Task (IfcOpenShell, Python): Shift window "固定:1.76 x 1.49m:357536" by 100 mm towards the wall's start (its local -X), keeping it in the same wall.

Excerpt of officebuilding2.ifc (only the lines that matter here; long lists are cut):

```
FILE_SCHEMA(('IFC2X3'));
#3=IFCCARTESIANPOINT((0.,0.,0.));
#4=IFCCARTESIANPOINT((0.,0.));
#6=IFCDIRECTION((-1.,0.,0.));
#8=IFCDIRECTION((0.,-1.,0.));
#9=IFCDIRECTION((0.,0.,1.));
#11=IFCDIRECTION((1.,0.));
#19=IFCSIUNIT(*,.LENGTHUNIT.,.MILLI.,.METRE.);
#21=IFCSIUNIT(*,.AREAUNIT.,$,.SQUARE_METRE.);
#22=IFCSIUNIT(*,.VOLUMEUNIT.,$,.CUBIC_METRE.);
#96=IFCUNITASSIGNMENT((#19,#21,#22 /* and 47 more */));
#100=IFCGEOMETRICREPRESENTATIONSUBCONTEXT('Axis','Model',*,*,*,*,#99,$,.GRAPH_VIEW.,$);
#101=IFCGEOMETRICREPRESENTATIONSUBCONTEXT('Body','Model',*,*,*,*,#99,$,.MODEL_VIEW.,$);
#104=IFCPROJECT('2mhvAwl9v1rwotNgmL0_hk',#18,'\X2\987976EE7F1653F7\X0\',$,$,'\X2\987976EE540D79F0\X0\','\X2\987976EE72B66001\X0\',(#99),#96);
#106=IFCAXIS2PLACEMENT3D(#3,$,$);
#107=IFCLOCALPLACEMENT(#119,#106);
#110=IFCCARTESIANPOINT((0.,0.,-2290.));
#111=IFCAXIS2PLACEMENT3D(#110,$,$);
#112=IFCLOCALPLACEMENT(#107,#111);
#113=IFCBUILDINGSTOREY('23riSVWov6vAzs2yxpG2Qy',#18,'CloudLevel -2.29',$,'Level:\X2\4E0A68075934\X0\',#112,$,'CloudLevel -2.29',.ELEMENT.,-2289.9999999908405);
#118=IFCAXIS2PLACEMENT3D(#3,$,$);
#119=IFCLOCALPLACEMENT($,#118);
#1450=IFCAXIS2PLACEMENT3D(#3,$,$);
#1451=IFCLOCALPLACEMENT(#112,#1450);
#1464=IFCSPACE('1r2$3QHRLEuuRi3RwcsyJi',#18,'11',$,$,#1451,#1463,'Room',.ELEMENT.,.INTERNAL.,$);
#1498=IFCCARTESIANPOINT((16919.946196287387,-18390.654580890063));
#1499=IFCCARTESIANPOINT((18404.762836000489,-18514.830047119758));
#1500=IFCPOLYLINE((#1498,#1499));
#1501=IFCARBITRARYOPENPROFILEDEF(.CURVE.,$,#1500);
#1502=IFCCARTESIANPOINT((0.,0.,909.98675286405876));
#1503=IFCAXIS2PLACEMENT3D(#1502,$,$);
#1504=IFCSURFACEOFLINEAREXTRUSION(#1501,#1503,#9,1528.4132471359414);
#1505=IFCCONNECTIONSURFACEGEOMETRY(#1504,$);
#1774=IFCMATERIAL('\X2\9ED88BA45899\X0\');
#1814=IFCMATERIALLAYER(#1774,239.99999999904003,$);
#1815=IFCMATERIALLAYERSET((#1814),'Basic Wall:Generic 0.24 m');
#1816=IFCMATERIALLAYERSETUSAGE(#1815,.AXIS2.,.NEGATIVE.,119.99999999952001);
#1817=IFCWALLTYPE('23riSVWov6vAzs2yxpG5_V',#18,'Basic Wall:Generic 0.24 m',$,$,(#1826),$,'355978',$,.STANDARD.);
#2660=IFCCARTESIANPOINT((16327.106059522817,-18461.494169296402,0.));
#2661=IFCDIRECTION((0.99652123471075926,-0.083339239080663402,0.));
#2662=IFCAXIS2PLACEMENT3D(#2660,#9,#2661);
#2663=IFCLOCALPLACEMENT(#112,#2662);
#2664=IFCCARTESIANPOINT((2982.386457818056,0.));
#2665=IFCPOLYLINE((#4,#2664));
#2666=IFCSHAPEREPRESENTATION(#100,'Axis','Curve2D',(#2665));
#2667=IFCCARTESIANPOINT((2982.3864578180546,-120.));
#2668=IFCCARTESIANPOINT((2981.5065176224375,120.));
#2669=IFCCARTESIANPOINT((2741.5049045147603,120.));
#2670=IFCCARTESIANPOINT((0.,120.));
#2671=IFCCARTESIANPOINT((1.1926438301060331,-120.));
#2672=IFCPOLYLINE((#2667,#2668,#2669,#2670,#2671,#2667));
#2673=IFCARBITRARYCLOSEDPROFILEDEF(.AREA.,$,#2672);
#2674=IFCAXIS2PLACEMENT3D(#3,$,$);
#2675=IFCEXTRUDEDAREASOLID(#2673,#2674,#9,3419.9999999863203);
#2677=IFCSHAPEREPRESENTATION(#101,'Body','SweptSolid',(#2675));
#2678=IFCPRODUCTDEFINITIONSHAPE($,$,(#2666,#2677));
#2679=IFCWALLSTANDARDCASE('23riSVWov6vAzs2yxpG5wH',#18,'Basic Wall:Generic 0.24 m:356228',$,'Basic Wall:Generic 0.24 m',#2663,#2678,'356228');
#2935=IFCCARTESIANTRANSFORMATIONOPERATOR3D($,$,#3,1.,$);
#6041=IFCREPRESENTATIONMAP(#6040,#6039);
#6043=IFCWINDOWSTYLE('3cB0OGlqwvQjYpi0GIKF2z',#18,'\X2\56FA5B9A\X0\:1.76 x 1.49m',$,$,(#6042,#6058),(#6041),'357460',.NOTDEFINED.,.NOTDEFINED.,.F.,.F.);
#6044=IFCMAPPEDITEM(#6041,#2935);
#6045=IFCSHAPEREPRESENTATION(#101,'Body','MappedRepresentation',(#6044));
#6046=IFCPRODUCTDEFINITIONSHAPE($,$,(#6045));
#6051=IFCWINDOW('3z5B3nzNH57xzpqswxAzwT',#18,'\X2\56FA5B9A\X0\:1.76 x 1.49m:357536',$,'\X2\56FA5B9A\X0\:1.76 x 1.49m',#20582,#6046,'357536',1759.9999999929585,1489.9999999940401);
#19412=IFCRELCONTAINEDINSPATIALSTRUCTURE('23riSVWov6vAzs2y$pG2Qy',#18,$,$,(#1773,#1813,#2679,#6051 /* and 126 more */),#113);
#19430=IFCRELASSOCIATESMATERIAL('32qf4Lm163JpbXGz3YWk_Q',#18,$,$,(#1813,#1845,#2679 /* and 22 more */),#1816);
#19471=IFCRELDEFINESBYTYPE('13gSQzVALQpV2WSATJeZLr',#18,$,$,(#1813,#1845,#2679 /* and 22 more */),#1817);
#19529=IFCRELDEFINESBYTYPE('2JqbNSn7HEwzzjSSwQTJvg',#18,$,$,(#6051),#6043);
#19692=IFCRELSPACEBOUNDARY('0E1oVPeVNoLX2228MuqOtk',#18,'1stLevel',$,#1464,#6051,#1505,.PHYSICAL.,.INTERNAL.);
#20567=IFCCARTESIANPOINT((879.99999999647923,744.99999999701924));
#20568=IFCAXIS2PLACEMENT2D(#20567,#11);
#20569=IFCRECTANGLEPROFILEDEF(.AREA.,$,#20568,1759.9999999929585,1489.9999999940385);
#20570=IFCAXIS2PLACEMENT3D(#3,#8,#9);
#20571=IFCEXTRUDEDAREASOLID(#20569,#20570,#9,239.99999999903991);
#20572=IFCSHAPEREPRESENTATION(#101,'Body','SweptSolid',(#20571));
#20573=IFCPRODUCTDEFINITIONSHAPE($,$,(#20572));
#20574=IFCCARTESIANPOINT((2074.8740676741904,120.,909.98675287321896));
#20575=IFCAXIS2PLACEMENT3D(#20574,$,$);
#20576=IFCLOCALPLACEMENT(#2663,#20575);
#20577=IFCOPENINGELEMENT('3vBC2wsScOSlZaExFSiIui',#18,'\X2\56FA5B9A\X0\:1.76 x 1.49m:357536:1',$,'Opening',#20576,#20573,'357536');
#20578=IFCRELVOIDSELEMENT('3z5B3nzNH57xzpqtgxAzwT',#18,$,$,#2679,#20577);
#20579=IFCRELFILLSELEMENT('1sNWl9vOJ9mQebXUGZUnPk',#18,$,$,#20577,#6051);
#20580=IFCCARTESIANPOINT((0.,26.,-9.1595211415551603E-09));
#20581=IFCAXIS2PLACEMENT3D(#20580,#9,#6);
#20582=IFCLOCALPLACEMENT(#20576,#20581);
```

```python
import numpy as np
import ifcopenshell
import ifcopenshell.api.geometry
import ifcopenshell.util.placement
import ifcopenshell.util.unit

model = ifcopenshell.open("officebuilding2.ifc")
unit_scale = ifcopenshell.util.unit.calculate_unit_scale(model)

window = model.by_guid("3z5B3nzNH57xzpqswxAzwT")
opening = window.FillsVoids[0].RelatingOpeningElement
wall = opening.VoidsElements[0].RelatingBuildingElement

wall_matrix = ifcopenshell.util.placement.get_local_placement(wall.ObjectPlacement)
shift = wall_matrix[:3, 0] * -0.1 / unit_scale
before = ifcopenshell.util.placement.get_local_placement(window.ObjectPlacement)[:3, 3].copy()

# The window is placed relative to its opening, so it follows when the opening moves.
matrix = ifcopenshell.util.placement.get_local_placement(opening.ObjectPlacement)
matrix[:3, 3] += shift
ifcopenshell.api.geometry.edit_object_placement(
    model, product=opening, matrix=matrix, is_si=False, should_transform_children=True
)

# Space boundary surfaces are stored in each space's coordinates; move them too.
for rel in window.ProvidesBoundaries:
    if not rel.ConnectionGeometry:
        continue
    surface = rel.ConnectionGeometry.SurfaceOnRelatingElement
    space_matrix = ifcopenshell.util.placement.get_local_placement(rel.RelatingSpace.ObjectPlacement)
    point = np.array(surface.Position.Location.Coordinates) + space_matrix[:3, :3].T @ shift
    surface.Position = model.createIfcAxis2Placement3D(
        model.createIfcCartesianPoint(point.tolist()), surface.Position.Axis, surface.Position.RefDirection
    )

after = ifcopenshell.util.placement.get_local_placement(window.ObjectPlacement)[:3, 3]
print("window moved by", (after - before).round(3) + 0.0)

model.write("officebuilding2_rev.ifc")
```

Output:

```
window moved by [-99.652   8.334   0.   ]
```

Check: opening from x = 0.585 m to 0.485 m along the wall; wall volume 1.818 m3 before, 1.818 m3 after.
